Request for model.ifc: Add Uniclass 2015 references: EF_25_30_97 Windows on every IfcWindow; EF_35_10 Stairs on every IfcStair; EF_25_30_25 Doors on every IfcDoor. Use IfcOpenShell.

First a look at what the model holds.

```python
import ifcopenshell

model = ifcopenshell.open("model.ifc")
print(model.schema)
print("classifications:", [c.Name for c in model.by_type("IfcClassification")])
for ifc_class in ("IfcDoor", "IfcRoof", "IfcStair", "IfcWall", "IfcWindow"):
    print(ifc_class, len(model.by_type(ifc_class)))
```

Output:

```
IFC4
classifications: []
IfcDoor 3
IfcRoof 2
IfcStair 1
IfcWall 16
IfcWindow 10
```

```python
import ifcopenshell
import ifcopenshell.api.classification

model = ifcopenshell.open("model.ifc")

system = ifcopenshell.api.classification.add_classification(model, classification="Uniclass 2015")

codes = {
    "IfcWindow": ("EF_25_30_97", "Windows"),
    "IfcStair": ("EF_35_10", "Stairs"),
    "IfcDoor": ("EF_25_30_25", "Doors"),
}
for ifc_class, (code, name) in codes.items():
    products = model.by_type(ifc_class)
    ifcopenshell.api.classification.add_reference(
        model, products=products, classification=system, identification=code, name=name
    )
    print(code, len(products))

model.write("model_updated.ifc")
```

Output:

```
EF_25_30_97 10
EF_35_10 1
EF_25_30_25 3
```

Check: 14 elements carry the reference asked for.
